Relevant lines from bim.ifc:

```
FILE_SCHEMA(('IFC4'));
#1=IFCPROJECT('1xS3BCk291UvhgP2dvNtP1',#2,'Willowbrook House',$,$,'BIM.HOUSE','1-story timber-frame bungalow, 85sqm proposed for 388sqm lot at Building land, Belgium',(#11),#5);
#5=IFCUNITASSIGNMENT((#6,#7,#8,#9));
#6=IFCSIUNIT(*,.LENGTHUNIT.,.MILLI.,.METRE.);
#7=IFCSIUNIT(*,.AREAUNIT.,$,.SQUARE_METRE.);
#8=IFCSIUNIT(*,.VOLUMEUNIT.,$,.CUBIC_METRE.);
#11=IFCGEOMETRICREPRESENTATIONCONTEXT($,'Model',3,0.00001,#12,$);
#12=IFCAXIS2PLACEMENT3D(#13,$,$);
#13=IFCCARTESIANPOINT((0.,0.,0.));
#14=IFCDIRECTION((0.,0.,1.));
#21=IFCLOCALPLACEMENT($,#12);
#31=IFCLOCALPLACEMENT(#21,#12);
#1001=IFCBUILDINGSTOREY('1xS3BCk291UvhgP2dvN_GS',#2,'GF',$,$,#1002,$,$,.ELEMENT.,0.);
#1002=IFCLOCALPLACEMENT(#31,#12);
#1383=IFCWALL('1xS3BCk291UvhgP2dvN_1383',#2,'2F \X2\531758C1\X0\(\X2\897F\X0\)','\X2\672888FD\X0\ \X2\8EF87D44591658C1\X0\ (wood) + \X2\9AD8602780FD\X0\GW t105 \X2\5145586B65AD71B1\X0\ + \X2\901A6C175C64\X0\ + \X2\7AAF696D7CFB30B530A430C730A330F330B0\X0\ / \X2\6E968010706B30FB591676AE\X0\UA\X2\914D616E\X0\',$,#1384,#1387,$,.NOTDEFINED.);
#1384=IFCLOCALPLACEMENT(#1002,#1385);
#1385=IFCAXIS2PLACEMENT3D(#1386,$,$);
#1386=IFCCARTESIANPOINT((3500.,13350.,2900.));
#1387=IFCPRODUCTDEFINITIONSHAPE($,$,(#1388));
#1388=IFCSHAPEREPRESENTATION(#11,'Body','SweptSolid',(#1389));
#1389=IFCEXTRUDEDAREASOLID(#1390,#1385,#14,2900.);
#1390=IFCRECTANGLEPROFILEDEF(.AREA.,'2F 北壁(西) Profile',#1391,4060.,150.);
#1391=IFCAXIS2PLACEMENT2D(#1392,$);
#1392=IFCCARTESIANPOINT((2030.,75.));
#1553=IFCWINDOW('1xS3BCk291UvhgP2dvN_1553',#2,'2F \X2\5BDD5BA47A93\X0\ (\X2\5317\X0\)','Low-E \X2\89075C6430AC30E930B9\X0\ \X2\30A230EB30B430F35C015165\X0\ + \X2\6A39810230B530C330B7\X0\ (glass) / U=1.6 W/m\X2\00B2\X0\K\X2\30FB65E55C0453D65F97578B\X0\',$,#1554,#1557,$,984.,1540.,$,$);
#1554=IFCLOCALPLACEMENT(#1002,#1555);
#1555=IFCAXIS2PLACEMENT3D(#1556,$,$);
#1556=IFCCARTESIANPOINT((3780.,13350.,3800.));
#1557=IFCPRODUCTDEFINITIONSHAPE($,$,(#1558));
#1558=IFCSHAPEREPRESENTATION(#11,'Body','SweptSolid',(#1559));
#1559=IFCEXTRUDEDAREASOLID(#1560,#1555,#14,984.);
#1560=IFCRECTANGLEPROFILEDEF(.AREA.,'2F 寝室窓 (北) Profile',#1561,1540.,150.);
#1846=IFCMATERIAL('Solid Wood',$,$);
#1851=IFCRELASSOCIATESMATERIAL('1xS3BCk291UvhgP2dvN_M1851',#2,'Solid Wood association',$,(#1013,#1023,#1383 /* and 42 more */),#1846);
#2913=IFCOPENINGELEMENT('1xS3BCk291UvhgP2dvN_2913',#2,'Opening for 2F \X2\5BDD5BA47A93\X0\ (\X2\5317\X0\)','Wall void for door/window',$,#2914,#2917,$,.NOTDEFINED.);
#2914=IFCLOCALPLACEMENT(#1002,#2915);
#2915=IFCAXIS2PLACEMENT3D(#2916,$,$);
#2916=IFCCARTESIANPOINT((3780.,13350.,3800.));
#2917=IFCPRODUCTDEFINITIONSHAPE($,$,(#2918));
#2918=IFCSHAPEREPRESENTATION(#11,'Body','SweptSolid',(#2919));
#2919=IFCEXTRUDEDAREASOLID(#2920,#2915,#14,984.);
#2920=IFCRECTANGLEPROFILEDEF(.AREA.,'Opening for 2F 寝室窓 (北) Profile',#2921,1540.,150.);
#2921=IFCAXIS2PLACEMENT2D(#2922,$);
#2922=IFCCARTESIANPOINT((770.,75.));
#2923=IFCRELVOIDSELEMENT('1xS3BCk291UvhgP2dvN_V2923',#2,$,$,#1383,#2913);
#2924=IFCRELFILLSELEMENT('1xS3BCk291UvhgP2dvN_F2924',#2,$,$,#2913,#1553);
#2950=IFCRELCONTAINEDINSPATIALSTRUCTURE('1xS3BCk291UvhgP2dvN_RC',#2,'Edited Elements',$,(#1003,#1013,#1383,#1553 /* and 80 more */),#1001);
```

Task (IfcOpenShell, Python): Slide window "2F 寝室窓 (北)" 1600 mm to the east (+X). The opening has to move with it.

```python
import ifcopenshell
import ifcopenshell.api.geometry
import ifcopenshell.util.placement
import ifcopenshell.util.unit

model = ifcopenshell.open("bim.ifc")
unit_scale = ifcopenshell.util.unit.calculate_unit_scale(model)

window = model.by_id(1553)
opening = window.FillsVoids[0].RelatingOpeningElement
wall = opening.VoidsElements[0].RelatingBuildingElement

wall_matrix = ifcopenshell.util.placement.get_local_placement(wall.ObjectPlacement)
shift = wall_matrix[:3, 0] * 1.6 / unit_scale
before = ifcopenshell.util.placement.get_local_placement(window.ObjectPlacement)[:3, 3].copy()

# The window is not placed relative to its opening, so move both.
for product in (opening, window):
    matrix = ifcopenshell.util.placement.get_local_placement(product.ObjectPlacement)
    matrix[:3, 3] += shift
    ifcopenshell.api.geometry.edit_object_placement(model, product=product, matrix=matrix, is_si=False)

after = ifcopenshell.util.placement.get_local_placement(window.ObjectPlacement)[:3, 3]
print("window moved by", (after - before).round(3) + 0.0)

model.write("bim_edited.ifc")
```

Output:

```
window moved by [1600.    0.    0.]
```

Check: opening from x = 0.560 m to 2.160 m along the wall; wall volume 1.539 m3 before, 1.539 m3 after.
